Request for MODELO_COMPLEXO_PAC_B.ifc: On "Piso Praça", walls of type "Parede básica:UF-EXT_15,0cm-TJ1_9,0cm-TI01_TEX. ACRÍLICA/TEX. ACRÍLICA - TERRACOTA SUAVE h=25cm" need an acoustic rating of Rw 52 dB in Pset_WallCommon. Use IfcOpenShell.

First a look at what the model holds.

```python
import ifcopenshell
import ifcopenshell.util.element

model = ifcopenshell.open("MODELO_COMPLEXO_PAC_B.ifc")
print(model.schema)
storey = next(s for s in model.by_type("IfcBuildingStorey") if s.Name == "Piso Praça")
walls = [e for e in ifcopenshell.util.element.get_decomposition(storey) if e.is_a("IfcWall")]
seen = {}
for e in walls:
    element_type = ifcopenshell.util.element.get_type(e)
    key = (element_type.Name if element_type != e and element_type else None, ifcopenshell.util.element.get_pset(e, "Pset_WallCommon", "AcousticRating"))
    seen[key] = seen.get(key, 0) + 1
for (name, value), count in sorted(seen.items(), key=str):
    print(count, "x", name, "|", value)
```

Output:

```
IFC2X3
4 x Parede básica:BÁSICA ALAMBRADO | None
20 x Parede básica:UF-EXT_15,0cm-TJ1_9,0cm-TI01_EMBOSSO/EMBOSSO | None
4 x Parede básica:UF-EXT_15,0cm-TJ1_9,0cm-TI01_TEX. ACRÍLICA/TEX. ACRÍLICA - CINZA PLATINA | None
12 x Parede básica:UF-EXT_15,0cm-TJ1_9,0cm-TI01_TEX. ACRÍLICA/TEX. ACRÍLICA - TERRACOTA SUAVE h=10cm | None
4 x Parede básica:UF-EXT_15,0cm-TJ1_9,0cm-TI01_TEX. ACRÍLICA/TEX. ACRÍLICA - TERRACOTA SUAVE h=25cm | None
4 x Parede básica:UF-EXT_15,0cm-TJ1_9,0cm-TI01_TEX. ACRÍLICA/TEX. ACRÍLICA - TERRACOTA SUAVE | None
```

```python
import ifcopenshell
import ifcopenshell.api.pset
import ifcopenshell.util.element

model = ifcopenshell.open("MODELO_COMPLEXO_PAC_B.ifc")

storey = next(s for s in model.by_type("IfcBuildingStorey") if s.Name == "Piso Praça")
walls = [e for e in ifcopenshell.util.element.get_decomposition(storey) if e.is_a("IfcWall")]

count = 0
for e in walls:
    element_type = ifcopenshell.util.element.get_type(e)
    if element_type in (None, e) or element_type.Name != "Parede básica:UF-EXT_15,0cm-TJ1_9,0cm-TI01_TEX. ACRÍLICA/TEX. ACRÍLICA - TERRACOTA SUAVE h=25cm":
        continue
    # add_pset returns the element's existing set when there is one.
    pset = ifcopenshell.api.pset.add_pset(model, product=e, name="Pset_WallCommon")
    ifcopenshell.api.pset.edit_pset(model, pset=pset, properties={"AcousticRating": "Rw 52 dB"})
    count += 1

print(count, "walls updated")

model.write("MODELO_COMPLEXO_PAC_B_v2.ifc")
```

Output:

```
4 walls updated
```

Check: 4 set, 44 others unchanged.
